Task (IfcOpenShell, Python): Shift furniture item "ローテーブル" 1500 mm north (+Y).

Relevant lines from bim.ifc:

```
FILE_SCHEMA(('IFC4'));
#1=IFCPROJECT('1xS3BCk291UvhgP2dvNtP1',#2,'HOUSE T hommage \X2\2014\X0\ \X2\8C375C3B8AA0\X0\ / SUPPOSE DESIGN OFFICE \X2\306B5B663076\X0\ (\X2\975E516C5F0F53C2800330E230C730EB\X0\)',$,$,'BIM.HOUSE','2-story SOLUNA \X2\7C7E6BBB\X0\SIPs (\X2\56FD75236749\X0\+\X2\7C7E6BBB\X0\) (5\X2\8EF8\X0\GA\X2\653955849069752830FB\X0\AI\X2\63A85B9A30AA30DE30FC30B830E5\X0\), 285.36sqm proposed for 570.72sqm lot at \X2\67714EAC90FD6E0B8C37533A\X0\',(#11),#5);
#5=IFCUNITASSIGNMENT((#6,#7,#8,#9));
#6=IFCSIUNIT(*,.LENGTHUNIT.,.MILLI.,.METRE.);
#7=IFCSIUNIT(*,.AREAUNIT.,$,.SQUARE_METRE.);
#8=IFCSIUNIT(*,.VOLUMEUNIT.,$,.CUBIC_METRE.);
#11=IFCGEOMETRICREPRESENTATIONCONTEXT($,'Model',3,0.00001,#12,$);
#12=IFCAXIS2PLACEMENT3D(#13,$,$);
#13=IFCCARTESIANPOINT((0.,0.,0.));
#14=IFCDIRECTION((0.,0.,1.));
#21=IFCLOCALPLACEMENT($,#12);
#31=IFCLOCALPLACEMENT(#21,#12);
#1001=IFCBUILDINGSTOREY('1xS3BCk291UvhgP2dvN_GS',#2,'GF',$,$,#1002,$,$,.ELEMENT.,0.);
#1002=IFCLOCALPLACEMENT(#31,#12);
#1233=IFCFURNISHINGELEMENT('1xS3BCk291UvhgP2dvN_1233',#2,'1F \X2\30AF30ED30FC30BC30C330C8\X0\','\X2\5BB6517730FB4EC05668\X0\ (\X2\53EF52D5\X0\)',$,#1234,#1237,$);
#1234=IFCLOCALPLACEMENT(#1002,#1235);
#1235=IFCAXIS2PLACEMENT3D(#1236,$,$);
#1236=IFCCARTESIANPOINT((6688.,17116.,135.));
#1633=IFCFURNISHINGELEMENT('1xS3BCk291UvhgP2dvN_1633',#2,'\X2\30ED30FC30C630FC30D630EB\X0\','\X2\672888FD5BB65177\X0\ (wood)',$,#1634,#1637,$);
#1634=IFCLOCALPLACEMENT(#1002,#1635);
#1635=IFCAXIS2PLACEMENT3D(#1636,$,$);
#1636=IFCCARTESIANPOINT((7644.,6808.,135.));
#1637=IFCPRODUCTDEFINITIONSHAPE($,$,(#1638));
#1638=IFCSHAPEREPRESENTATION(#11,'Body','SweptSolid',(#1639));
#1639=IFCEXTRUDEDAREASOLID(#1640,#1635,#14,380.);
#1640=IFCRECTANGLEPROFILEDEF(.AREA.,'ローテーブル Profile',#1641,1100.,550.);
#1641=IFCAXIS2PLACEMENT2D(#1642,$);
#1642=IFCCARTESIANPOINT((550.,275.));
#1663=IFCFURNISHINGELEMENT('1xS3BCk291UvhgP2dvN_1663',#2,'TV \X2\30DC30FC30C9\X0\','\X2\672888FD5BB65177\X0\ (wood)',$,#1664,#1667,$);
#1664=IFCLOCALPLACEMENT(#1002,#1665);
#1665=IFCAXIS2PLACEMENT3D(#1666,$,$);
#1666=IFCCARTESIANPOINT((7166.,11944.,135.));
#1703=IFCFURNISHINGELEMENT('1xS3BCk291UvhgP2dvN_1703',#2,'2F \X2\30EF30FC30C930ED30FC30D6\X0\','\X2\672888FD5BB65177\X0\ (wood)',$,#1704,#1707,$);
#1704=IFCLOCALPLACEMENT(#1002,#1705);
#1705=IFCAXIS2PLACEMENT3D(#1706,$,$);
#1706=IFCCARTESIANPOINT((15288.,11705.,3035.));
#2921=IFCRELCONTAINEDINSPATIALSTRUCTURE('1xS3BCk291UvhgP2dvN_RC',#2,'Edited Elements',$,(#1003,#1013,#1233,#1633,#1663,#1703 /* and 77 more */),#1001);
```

```python
import ifcopenshell
import ifcopenshell.api.geometry
import ifcopenshell.util.placement
import ifcopenshell.util.unit

model = ifcopenshell.open("bim.ifc")
unit_scale = ifcopenshell.util.unit.calculate_unit_scale(model)

item = model.by_guid("1xS3BCk291UvhgP2dvN_1633")
matrix = ifcopenshell.util.placement.get_local_placement(item.ObjectPlacement)
matrix[1, 3] += 1.5 / unit_scale
ifcopenshell.api.geometry.edit_object_placement(model, product=item, matrix=matrix, is_si=False)

print(ifcopenshell.util.placement.get_local_placement(item.ObjectPlacement).round(3) + 0.0)

model.write("bim_edited.ifc")
```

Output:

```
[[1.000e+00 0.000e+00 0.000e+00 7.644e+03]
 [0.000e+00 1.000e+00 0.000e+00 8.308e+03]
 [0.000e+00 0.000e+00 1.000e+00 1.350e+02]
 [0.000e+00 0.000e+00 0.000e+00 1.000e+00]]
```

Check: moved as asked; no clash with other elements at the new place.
